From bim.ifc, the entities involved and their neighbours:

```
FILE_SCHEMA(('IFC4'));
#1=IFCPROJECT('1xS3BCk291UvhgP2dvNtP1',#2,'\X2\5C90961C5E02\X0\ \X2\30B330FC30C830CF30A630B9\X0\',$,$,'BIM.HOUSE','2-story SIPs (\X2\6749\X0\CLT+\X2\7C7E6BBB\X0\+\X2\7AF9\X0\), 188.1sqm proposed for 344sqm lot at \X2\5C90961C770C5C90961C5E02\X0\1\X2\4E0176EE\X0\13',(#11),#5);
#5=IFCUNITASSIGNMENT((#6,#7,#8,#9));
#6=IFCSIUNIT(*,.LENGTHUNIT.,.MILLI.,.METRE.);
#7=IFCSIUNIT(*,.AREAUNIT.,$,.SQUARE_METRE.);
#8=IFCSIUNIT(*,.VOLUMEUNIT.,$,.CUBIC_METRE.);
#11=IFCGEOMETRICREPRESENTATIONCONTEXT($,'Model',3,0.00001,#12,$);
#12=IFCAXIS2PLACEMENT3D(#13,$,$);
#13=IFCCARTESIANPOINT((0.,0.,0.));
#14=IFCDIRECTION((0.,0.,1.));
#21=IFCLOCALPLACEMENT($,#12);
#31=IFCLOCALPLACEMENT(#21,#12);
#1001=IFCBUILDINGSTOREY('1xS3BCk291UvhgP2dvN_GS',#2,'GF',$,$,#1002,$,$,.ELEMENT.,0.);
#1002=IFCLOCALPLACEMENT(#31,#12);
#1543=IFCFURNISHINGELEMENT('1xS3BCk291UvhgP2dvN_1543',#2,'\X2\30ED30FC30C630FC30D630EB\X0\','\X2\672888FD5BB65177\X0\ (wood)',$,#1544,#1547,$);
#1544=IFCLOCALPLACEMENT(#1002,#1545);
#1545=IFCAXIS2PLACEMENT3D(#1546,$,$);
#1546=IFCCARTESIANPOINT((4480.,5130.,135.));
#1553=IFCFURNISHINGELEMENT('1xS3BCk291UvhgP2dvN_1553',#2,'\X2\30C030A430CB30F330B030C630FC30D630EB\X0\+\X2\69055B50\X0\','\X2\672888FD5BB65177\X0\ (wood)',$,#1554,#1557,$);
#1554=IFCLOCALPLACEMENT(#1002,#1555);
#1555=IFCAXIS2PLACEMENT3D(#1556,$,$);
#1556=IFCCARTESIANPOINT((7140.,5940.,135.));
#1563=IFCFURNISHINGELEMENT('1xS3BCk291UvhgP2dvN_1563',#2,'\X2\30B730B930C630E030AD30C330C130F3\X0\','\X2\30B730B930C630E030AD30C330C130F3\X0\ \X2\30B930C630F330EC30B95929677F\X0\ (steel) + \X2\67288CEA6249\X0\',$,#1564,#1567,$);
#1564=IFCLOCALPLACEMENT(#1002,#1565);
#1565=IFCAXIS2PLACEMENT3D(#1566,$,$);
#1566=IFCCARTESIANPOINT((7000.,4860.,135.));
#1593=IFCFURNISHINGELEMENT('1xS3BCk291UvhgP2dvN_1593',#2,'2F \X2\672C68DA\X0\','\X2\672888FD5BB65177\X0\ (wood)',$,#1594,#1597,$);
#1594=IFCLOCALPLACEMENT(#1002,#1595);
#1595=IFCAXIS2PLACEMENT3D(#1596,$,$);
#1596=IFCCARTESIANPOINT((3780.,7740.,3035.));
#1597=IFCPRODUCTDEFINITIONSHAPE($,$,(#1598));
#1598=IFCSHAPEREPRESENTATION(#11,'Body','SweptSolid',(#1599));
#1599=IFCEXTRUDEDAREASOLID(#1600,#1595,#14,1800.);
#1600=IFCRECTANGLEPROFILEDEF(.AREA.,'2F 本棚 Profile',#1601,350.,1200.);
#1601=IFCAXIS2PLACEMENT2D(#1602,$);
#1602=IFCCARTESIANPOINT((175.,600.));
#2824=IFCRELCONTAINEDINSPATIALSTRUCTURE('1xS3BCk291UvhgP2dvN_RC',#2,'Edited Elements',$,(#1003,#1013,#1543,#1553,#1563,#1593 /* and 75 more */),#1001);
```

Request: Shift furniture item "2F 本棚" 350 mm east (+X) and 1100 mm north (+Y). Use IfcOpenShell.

```python
import ifcopenshell
import ifcopenshell.api.geometry
import ifcopenshell.util.placement
import ifcopenshell.util.unit

model = ifcopenshell.open("bim.ifc")
unit_scale = ifcopenshell.util.unit.calculate_unit_scale(model)

item = model.by_guid("1xS3BCk291UvhgP2dvN_1593")
matrix = ifcopenshell.util.placement.get_local_placement(item.ObjectPlacement)
matrix[0, 3] += 0.35 / unit_scale
matrix[1, 3] += 1.1 / unit_scale
ifcopenshell.api.geometry.edit_object_placement(model, product=item, matrix=matrix, is_si=False)

print(ifcopenshell.util.placement.get_local_placement(item.ObjectPlacement).round(3) + 0.0)

model.write("bim_v2.ifc")
```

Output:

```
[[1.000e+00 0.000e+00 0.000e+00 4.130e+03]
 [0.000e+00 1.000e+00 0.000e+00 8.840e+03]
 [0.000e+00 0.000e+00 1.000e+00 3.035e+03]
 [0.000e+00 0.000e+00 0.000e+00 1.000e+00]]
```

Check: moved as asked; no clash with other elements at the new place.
